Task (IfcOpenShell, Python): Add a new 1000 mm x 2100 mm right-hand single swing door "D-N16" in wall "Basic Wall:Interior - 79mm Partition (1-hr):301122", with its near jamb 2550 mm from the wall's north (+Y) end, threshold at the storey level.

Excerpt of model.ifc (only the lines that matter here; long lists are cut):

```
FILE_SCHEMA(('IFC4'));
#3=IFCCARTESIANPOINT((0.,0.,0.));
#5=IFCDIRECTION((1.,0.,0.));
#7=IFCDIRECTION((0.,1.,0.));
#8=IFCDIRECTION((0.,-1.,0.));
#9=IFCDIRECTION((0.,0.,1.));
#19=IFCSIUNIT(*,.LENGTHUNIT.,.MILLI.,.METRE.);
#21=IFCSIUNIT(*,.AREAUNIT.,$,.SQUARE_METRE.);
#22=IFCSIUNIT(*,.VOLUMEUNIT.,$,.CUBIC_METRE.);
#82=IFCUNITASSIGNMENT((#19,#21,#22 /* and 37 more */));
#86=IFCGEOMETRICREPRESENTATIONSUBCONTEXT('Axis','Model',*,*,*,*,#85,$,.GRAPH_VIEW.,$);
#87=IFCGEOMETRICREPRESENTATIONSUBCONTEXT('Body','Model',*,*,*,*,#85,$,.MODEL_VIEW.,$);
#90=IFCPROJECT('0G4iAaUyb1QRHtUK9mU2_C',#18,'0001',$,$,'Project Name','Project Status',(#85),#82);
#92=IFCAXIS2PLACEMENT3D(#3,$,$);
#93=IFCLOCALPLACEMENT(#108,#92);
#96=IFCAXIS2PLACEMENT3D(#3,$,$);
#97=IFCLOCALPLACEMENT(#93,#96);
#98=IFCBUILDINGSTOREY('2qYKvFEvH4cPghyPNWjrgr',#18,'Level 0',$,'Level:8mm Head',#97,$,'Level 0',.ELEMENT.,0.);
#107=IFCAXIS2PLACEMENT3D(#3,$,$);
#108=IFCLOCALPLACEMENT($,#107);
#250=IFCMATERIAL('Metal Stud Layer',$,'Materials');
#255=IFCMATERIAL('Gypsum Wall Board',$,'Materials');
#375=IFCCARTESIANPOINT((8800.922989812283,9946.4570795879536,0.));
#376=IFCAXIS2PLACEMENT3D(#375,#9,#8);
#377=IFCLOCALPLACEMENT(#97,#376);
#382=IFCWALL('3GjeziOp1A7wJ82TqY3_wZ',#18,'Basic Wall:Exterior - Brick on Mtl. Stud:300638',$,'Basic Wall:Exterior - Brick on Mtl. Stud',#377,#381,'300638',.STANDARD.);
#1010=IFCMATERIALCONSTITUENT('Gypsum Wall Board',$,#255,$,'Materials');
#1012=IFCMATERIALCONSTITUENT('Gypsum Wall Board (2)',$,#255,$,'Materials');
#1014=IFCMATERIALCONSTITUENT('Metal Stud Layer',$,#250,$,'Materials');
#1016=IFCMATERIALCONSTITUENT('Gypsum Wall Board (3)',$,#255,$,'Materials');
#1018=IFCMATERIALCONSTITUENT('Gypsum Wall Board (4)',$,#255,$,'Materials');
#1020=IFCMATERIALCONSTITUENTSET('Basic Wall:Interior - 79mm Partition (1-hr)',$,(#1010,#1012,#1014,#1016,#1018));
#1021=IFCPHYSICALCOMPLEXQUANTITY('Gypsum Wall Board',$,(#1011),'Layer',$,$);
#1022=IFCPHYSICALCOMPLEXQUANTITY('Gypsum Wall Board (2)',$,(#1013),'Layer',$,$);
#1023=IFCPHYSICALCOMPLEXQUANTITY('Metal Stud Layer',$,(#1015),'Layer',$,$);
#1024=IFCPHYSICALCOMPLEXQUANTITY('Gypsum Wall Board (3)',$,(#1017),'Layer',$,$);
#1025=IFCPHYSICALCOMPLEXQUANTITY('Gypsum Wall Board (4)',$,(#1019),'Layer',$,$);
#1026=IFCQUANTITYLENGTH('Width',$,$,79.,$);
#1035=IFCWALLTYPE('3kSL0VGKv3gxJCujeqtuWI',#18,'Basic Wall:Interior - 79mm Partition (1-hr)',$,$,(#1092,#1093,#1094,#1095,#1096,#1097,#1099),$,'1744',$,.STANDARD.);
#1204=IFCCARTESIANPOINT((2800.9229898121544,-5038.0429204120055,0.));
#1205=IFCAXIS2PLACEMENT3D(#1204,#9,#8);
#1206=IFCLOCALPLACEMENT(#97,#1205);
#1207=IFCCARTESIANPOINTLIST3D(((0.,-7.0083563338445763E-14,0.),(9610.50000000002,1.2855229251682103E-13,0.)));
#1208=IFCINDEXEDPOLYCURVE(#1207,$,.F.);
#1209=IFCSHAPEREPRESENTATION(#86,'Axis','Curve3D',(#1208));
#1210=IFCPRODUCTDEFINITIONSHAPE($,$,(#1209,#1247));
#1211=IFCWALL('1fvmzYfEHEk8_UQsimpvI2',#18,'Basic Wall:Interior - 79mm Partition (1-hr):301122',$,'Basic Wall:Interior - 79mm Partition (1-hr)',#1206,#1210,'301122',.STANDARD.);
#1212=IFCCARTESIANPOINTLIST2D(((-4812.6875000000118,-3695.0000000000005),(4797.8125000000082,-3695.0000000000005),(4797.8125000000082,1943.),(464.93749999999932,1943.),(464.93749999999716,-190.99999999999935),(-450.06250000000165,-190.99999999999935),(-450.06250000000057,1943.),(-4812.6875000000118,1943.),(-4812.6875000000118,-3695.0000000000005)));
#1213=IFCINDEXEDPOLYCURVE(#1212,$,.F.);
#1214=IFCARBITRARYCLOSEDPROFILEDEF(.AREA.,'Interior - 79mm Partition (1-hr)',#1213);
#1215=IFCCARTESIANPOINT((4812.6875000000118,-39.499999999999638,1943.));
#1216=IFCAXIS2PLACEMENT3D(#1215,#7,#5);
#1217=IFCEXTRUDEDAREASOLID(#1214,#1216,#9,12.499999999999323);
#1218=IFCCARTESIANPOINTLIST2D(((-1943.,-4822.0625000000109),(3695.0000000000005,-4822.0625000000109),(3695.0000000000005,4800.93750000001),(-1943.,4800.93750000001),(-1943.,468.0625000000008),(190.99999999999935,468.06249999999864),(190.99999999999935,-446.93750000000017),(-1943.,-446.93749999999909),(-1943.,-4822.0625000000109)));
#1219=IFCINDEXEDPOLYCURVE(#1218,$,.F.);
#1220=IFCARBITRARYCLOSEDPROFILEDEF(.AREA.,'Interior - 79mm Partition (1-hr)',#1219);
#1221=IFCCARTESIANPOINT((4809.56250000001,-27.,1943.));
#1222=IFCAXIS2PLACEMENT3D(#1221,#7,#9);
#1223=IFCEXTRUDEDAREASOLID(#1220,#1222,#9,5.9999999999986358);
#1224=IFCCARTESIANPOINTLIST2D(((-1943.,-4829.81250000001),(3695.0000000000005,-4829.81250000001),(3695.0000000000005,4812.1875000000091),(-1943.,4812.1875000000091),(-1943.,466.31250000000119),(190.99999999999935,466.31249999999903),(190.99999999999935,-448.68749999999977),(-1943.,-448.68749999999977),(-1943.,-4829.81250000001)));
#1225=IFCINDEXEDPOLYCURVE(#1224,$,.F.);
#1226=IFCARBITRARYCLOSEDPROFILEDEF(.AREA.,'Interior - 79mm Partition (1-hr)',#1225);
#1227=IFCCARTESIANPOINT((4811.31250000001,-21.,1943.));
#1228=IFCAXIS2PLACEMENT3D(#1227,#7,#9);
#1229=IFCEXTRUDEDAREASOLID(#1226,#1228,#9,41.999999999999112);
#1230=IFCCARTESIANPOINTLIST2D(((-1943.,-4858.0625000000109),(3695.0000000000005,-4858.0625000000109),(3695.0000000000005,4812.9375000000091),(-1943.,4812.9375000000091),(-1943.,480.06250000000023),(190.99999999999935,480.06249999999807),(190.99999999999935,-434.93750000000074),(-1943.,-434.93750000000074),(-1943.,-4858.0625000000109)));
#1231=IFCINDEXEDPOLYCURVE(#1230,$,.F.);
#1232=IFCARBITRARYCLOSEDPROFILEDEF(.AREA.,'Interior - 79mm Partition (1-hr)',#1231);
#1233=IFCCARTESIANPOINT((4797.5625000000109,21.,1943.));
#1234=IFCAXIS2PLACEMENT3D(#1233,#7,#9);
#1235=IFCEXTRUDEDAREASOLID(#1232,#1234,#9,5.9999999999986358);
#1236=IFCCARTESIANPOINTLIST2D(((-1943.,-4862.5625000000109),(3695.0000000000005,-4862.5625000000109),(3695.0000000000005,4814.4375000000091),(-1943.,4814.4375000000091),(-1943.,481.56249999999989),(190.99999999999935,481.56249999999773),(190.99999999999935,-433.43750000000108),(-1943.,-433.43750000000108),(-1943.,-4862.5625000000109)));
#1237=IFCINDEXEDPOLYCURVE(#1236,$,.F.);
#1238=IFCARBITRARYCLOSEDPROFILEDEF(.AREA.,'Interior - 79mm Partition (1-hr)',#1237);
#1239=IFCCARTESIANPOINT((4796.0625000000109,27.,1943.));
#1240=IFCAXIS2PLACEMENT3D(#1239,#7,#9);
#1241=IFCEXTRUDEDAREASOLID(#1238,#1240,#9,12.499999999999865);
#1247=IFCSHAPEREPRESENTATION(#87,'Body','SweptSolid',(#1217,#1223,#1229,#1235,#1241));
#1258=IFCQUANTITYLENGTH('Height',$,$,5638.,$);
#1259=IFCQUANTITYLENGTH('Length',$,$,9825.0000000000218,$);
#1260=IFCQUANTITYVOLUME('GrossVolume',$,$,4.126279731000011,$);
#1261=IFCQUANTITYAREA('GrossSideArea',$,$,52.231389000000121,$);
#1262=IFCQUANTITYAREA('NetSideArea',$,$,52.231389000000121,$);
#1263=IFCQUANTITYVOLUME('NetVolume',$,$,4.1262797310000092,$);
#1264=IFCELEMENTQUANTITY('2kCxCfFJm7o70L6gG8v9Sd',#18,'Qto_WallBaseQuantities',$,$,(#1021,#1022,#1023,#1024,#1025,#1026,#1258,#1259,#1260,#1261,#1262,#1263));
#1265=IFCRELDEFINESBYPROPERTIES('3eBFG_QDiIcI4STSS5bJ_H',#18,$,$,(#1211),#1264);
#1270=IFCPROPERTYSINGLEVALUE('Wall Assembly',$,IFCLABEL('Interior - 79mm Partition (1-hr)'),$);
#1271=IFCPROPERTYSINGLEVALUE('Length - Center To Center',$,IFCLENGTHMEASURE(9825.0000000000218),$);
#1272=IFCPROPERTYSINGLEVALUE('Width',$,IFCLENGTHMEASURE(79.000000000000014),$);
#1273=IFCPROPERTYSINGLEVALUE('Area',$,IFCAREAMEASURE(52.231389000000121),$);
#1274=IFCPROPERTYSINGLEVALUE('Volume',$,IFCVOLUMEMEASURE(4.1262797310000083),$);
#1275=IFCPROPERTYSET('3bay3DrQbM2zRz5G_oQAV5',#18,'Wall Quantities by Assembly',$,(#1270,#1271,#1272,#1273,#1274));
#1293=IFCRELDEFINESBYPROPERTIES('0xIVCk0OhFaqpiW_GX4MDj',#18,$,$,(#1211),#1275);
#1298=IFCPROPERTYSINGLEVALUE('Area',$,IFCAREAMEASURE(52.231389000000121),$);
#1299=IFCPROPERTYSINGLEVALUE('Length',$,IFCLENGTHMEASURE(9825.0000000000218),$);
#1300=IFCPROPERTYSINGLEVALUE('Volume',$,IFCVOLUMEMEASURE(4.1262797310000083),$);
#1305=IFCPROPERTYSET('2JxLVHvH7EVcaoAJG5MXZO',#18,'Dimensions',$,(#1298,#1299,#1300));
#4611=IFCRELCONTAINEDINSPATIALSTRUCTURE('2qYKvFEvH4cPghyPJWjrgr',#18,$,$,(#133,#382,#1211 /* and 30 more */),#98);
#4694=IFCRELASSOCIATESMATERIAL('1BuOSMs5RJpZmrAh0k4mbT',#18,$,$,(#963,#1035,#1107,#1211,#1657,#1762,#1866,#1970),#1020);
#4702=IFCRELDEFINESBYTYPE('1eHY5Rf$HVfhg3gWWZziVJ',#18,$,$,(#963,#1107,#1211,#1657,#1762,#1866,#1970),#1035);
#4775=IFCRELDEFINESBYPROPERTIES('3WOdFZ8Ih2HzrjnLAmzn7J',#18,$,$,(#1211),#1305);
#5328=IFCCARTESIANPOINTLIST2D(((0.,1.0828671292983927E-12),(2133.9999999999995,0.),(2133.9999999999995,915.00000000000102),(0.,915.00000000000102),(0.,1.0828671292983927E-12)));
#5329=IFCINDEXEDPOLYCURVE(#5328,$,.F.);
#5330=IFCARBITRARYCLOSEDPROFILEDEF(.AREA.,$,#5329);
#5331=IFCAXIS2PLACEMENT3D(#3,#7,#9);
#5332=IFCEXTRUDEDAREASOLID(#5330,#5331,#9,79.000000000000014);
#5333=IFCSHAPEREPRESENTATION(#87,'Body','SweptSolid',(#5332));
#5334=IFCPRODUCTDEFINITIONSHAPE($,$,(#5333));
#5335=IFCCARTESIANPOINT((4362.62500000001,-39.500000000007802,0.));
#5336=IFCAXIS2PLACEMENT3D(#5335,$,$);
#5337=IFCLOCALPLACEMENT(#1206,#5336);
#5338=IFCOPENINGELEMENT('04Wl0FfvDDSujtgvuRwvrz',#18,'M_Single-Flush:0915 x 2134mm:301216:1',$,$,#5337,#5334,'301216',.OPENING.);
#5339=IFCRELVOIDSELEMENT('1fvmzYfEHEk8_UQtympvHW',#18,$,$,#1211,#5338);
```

```python
import numpy as np
import ifcopenshell
import ifcopenshell.api.feature
import ifcopenshell.api.geometry
import ifcopenshell.api.pset
import ifcopenshell.api.root
import ifcopenshell.api.spatial
import ifcopenshell.geom
import ifcopenshell.util.element
import ifcopenshell.util.placement
import ifcopenshell.util.representation
import ifcopenshell.util.shape
import ifcopenshell.util.unit

model = ifcopenshell.open("model.ifc")
unit_scale = ifcopenshell.util.unit.calculate_unit_scale(model)
area_scale = ifcopenshell.util.unit.calculate_unit_scale(model, "AREAUNIT")
volume_scale = ifcopenshell.util.unit.calculate_unit_scale(model, "VOLUMEUNIT")
settings = ifcopenshell.geom.settings()


def volume(element):
    """Net volume in cubic metres, openings subtracted."""
    shape = ifcopenshell.geom.create_shape(settings, element)
    return ifcopenshell.util.shape.get_volume(shape.geometry)


wall = model.by_guid("1fvmzYfEHEk8_UQsimpvI2")
storey = ifcopenshell.util.element.get_container(wall, ifc_class="IfcBuildingStorey")
context = ifcopenshell.util.representation.get_context(model, "Model", "Body", "MODEL_VIEW")
before = volume(wall)

width, height, from_end, sill = 1, 2.1, 2.55, 0.0  # metres

# The wall runs along its own X axis, and the end named is its -X end.
wall_shape = ifcopenshell.geom.create_shape(settings, wall)
x, y, z = ifcopenshell.util.shape.get_vertices(wall_shape.geometry).T
start = x.min() + from_end
face, thickness = float(y.min()), float(y.max() - y.min())
wall_matrix = ifcopenshell.util.placement.get_local_placement(wall.ObjectPlacement)
level = ifcopenshell.util.placement.get_local_placement(storey.ObjectPlacement)[2, 3]


def in_wall(x, y):
    """Placement at x, y metres in the wall's axes, at sill height."""
    matrix = wall_matrix.copy()
    matrix[:, 3] = wall_matrix @ np.array([x / unit_scale, y / unit_scale, 0.0, 1.0])
    matrix[2, 3] = level + sill / unit_scale
    return matrix


# Opening: a box that overshoots both wall faces by 50 mm.
opening = ifcopenshell.api.root.create_entity(model, ifc_class="IfcOpeningElement", predefined_type="OPENING")
box = ifcopenshell.api.geometry.add_wall_representation(
    model, context=context, length=width, height=height, thickness=thickness + 0.1
)
ifcopenshell.api.geometry.assign_representation(model, product=opening, representation=box)
ifcopenshell.api.geometry.edit_object_placement(model, product=opening, matrix=in_wall(start, face - 0.05), is_si=False)
ifcopenshell.api.feature.add_feature(model, feature=opening, element=wall)

door = ifcopenshell.api.root.create_entity(model, ifc_class="IfcDoor", name="D-N16", predefined_type="DOOR")
door.OverallWidth, door.OverallHeight = width / unit_scale, height / unit_scale
door.OperationType = "SINGLE_SWING_RIGHT"
body = ifcopenshell.api.geometry.add_door_representation(
    model,
    context=context,
    overall_width=door.OverallWidth,
    overall_height=door.OverallHeight,
    operation_type="SINGLE_SWING_RIGHT",
    lining_properties={"LiningDepth": thickness / unit_scale, "ThresholdDepth": thickness / unit_scale},
)
ifcopenshell.api.geometry.assign_representation(model, product=door, representation=body)
ifcopenshell.api.spatial.assign_container(model, products=[door], relating_structure=storey)
ifcopenshell.api.feature.add_filling(model, opening=opening, element=door)

# The lining spans the wall, so the door starts at the wall face.
ifcopenshell.api.geometry.edit_object_placement(model, product=door, matrix=in_wall(start, face), is_si=False)

after = volume(wall)

# Update the wall's stored quantities.
qto = model.by_id(ifcopenshell.util.element.get_pset(wall, "Qto_WallBaseQuantities", should_inherit=False)["id"])
ifcopenshell.api.pset.edit_qto(model, qto=qto, properties={
    "NetSideArea": after / thickness / area_scale,
    "NetVolume": after / volume_scale,
})
pset = model.by_id(ifcopenshell.util.element.get_pset(wall, "Wall Quantities by Assembly", should_inherit=False)["id"])
ifcopenshell.api.pset.edit_pset(model, pset=pset, properties={
    "Area": model.create_entity("IfcAreaMeasure", after / thickness / area_scale),
    "Volume": model.create_entity("IfcVolumeMeasure", after / volume_scale),
})
pset = model.by_id(ifcopenshell.util.element.get_pset(wall, "Dimensions", should_inherit=False)["id"])
ifcopenshell.api.pset.edit_pset(model, pset=pset, properties={
    "Area": model.create_entity("IfcAreaMeasure", after / thickness / area_scale),
    "Volume": model.create_entity("IfcVolumeMeasure", after / volume_scale),
})

print(f"wall volume {before:.3f} -> {after:.3f} m3")

model.write("model_rev.ifc")
```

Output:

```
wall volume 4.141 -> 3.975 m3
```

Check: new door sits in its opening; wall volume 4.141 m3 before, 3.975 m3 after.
